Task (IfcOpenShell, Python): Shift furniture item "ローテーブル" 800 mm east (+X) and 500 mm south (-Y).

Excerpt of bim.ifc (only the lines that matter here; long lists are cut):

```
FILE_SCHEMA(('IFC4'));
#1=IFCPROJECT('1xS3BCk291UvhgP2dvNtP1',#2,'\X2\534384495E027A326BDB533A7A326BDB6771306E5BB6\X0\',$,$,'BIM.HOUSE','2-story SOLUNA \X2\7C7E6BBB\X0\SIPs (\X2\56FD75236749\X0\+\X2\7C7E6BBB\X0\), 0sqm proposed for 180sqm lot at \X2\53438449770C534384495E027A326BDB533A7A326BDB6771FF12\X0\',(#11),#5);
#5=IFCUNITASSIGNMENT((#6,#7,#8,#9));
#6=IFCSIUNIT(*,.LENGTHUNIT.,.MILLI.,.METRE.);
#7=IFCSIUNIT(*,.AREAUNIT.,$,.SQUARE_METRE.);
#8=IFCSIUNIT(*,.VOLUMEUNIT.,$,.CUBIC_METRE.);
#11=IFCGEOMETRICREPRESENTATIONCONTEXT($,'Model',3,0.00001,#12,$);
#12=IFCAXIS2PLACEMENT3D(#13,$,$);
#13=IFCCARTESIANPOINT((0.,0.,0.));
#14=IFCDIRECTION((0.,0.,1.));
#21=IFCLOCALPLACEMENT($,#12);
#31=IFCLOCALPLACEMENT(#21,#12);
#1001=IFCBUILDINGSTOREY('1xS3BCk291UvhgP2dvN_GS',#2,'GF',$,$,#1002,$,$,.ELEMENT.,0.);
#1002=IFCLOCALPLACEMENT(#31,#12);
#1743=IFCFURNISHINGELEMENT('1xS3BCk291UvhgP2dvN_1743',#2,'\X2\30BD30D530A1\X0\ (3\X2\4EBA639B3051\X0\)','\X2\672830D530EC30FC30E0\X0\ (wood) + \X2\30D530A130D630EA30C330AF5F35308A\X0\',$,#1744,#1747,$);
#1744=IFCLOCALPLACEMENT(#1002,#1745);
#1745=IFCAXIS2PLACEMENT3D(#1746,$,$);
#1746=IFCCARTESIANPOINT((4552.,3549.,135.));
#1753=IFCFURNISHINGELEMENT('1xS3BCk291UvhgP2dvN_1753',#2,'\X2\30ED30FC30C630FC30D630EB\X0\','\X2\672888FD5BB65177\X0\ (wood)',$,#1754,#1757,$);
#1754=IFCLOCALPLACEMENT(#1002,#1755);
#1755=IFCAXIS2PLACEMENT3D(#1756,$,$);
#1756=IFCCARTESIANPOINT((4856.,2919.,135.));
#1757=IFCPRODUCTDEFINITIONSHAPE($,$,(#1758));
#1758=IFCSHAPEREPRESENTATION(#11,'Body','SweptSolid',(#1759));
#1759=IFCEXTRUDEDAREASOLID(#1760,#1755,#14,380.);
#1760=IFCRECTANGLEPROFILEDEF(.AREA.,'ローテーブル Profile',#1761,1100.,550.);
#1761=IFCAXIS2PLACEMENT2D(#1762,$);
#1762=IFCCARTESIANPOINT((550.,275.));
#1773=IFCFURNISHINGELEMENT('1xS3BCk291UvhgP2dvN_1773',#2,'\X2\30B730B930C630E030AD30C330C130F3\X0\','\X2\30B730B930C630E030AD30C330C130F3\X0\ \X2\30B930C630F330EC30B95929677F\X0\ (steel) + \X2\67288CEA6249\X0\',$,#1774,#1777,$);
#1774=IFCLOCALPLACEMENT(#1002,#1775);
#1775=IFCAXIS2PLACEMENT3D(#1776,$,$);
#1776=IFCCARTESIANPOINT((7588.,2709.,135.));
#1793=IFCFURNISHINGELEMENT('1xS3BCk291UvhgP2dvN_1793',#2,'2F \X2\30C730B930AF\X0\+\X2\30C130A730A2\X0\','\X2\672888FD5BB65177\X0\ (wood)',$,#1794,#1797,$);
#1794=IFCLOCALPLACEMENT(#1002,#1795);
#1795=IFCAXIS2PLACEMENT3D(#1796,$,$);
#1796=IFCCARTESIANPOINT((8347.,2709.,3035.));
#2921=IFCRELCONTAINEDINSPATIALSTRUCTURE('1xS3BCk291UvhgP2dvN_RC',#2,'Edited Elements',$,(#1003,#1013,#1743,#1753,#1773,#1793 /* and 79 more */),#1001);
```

```python
import ifcopenshell
import ifcopenshell.api.geometry
import ifcopenshell.util.placement

model = ifcopenshell.open("bim.ifc")

item = model.by_id(1753)
matrix = ifcopenshell.util.placement.get_local_placement(item.ObjectPlacement)
matrix[0, 3] += 800.0
matrix[1, 3] -= 500.0
ifcopenshell.api.geometry.edit_object_placement(model, product=item, matrix=matrix, is_si=False)

print(ifcopenshell.util.placement.get_local_placement(item.ObjectPlacement).round(3) + 0.0)

model.write("bim-out.ifc")
```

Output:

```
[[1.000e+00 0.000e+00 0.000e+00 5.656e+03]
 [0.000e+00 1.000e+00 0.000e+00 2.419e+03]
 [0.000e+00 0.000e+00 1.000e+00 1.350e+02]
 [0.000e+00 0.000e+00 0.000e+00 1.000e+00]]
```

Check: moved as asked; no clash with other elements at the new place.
